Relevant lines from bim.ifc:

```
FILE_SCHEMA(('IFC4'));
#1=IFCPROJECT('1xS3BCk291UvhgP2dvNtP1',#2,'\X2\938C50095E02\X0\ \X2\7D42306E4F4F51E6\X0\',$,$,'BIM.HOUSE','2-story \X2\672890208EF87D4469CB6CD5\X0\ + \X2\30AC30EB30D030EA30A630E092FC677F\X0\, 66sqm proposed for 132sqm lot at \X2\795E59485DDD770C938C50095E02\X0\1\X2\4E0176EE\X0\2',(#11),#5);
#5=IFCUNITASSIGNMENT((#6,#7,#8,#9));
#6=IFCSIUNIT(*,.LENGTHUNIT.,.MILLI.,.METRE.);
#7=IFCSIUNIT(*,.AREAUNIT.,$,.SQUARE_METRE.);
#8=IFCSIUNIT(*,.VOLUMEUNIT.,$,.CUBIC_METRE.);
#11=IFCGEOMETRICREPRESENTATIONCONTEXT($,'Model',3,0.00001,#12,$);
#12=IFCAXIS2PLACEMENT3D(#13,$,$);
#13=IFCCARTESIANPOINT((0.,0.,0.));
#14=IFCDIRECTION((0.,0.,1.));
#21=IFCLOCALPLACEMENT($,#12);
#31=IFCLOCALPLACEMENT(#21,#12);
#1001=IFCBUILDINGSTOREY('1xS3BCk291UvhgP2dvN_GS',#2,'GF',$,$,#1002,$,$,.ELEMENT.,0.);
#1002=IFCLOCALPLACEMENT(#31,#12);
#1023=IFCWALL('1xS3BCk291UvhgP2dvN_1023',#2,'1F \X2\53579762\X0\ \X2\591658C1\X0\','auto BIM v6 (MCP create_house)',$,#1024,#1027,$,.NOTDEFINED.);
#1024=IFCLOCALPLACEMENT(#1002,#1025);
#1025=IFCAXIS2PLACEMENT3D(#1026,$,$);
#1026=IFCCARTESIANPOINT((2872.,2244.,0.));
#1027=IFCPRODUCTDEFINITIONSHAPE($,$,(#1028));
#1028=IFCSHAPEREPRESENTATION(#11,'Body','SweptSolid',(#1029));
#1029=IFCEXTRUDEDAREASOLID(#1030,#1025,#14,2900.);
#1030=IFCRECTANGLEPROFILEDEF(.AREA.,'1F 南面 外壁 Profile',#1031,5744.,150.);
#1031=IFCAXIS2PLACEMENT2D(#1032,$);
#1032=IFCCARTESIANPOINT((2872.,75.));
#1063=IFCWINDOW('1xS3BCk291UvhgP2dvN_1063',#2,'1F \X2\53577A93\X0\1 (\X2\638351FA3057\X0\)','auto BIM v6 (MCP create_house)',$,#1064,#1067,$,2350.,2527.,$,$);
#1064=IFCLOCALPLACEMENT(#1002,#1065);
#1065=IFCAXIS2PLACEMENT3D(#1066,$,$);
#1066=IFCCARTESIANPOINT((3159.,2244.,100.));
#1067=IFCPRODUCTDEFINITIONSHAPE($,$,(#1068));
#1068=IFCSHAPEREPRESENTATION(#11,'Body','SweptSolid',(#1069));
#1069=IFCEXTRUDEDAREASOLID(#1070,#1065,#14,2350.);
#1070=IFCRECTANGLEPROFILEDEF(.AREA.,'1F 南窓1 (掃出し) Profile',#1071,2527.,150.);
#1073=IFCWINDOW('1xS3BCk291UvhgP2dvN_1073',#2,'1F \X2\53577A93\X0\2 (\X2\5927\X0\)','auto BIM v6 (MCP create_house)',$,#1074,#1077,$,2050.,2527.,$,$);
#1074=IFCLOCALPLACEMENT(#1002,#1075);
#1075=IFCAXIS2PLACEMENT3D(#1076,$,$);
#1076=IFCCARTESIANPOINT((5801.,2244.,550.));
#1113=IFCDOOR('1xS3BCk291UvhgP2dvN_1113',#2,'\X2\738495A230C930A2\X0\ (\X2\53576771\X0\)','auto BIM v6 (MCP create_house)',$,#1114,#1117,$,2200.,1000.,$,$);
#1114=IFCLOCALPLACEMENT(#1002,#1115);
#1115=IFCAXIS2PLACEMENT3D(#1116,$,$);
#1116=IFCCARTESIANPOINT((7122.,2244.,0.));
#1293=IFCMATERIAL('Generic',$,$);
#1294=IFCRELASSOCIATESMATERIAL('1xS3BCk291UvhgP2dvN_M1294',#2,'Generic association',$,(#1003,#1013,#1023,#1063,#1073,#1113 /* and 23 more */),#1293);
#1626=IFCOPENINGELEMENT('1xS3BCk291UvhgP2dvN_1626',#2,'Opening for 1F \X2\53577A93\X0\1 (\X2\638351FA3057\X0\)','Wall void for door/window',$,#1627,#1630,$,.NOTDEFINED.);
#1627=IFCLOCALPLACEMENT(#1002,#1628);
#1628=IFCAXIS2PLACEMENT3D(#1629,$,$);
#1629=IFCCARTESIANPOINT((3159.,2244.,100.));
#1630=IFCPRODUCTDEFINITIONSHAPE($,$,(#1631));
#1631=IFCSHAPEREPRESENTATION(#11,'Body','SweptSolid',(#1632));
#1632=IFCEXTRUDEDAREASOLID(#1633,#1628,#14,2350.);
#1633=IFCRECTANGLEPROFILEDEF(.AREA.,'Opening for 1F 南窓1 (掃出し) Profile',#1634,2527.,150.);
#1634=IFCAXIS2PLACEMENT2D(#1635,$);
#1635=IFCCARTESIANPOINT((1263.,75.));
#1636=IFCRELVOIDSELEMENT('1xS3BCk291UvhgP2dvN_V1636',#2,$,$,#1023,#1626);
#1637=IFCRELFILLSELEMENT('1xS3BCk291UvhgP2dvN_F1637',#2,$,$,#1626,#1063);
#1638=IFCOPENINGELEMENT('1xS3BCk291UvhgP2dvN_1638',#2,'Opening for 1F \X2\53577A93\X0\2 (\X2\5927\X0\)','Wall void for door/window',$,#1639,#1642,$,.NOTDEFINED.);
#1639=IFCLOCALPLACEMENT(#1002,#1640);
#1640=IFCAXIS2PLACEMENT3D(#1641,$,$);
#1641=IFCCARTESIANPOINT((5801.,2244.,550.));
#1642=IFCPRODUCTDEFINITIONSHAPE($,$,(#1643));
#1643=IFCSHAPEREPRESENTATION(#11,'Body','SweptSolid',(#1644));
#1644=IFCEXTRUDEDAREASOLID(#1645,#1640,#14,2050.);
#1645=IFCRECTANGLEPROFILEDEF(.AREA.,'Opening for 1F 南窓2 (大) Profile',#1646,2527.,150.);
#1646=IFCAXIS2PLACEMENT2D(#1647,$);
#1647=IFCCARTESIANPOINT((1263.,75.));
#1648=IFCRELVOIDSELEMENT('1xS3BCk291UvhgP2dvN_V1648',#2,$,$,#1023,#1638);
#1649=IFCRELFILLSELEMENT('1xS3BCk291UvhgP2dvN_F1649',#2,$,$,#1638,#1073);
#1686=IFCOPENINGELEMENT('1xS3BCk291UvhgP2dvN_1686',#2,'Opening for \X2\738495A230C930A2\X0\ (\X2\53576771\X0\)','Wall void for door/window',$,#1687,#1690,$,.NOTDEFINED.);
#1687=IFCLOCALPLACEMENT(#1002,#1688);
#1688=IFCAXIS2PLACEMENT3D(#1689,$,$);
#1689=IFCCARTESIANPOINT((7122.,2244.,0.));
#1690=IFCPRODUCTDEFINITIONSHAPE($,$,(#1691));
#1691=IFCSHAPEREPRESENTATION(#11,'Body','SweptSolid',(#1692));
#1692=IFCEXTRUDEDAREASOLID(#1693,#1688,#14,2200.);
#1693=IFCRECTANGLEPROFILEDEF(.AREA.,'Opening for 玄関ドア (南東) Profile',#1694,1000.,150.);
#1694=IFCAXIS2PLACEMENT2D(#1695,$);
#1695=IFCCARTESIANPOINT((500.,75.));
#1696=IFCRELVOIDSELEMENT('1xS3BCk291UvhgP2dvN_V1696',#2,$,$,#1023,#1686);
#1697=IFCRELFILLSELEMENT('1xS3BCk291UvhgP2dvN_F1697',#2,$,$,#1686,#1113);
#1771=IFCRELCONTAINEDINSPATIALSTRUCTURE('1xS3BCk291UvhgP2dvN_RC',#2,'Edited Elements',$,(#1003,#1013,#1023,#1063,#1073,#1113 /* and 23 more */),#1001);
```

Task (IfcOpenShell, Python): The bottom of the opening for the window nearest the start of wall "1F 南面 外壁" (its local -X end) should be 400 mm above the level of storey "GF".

```python
import numpy as np
import ifcopenshell
import ifcopenshell.api.geometry
import ifcopenshell.geom
import ifcopenshell.util.element
import ifcopenshell.util.placement
import ifcopenshell.util.shape
import ifcopenshell.util.unit

model = ifcopenshell.open("bim.ifc")
unit_scale = ifcopenshell.util.unit.calculate_unit_scale(model)

window = model.by_id(1063)
opening = window.FillsVoids[0].RelatingOpeningElement
storey = ifcopenshell.util.element.get_container(window, ifc_class="IfcBuildingStorey")
level = ifcopenshell.util.placement.get_local_placement(storey.ObjectPlacement)[2, 3]

# The opening's origin need not be at the sill, so measure its lowest point.
shape = ifcopenshell.geom.create_shape(ifcopenshell.geom.settings(), opening)
bottom = ifcopenshell.util.shape.get_shape_bottom_elevation(shape, shape.geometry) / unit_scale
dz = level + 400.0 - bottom

shift = np.array([0.0, 0.0, dz])
# The window is not placed relative to its opening, so move both.
for product in (opening, window):
    matrix = ifcopenshell.util.placement.get_local_placement(product.ObjectPlacement)
    matrix[:3, 3] += shift
    ifcopenshell.api.geometry.edit_object_placement(model, product=product, matrix=matrix, is_si=False)

print(f"moved by {dz * unit_scale:+.3f} m")

model.write("bim_rev.ifc")
```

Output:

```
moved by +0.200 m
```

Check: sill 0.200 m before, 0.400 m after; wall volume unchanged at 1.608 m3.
